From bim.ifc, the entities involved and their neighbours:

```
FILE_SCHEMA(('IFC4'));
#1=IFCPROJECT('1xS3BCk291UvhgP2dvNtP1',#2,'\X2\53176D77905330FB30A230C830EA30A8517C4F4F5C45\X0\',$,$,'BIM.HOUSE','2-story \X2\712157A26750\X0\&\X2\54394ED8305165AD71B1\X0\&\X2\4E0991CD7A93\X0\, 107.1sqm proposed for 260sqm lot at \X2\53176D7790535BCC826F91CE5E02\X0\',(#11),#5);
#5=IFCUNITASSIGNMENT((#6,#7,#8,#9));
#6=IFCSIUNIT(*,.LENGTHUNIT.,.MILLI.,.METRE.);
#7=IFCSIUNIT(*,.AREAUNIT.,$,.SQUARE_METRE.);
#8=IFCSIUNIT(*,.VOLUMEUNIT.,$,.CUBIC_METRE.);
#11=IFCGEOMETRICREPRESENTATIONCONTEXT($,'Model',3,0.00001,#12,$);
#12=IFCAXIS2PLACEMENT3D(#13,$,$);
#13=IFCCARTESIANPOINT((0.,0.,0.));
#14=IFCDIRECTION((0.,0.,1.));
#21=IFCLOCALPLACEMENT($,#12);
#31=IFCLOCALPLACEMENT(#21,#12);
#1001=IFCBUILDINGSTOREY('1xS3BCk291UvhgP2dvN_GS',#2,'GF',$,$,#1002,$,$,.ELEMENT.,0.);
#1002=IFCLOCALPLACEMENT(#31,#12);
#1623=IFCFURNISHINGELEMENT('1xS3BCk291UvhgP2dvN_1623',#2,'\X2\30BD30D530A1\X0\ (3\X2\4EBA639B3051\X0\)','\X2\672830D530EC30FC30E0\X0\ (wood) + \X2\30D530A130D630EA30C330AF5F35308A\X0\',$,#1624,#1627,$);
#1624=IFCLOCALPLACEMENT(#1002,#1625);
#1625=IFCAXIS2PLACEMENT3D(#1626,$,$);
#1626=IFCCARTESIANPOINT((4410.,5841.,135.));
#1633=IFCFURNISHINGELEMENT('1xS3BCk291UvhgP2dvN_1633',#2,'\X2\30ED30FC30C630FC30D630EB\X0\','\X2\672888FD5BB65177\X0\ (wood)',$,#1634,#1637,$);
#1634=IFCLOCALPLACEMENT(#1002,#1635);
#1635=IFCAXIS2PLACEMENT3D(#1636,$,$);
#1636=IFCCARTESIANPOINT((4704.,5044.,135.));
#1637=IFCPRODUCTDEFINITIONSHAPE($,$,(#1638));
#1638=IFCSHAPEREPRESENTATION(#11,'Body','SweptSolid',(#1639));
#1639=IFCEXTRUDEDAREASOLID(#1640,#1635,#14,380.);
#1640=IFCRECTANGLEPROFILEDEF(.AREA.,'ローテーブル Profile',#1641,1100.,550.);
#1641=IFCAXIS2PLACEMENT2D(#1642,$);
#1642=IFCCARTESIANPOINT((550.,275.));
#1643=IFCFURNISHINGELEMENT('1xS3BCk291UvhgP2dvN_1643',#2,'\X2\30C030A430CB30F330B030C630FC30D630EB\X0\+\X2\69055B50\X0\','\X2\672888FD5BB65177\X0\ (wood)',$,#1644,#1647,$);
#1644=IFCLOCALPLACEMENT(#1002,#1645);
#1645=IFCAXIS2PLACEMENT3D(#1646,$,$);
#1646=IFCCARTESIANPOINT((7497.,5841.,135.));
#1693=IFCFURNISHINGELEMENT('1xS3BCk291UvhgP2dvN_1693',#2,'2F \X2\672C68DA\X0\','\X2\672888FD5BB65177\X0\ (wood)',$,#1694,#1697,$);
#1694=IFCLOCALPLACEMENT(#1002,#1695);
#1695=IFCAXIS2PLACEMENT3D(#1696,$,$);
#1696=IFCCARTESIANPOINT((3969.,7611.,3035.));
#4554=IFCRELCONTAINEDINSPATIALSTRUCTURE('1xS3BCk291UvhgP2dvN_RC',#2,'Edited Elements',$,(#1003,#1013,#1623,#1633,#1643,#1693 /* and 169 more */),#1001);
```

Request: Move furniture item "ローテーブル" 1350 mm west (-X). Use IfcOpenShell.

```python
import ifcopenshell
import ifcopenshell.api.geometry
import ifcopenshell.util.placement
import ifcopenshell.util.unit

model = ifcopenshell.open("bim.ifc")
unit_scale = ifcopenshell.util.unit.calculate_unit_scale(model)

item = model.by_guid("1xS3BCk291UvhgP2dvN_1633")
matrix = ifcopenshell.util.placement.get_local_placement(item.ObjectPlacement)
matrix[0, 3] -= 1.35 / unit_scale
ifcopenshell.api.geometry.edit_object_placement(model, product=item, matrix=matrix, is_si=False)

print(ifcopenshell.util.placement.get_local_placement(item.ObjectPlacement).round(3) + 0.0)

model.write("bim_updated.ifc")
```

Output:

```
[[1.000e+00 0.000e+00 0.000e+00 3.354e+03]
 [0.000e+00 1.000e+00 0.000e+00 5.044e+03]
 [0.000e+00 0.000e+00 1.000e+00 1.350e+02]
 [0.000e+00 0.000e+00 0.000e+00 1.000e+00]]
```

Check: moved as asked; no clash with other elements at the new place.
